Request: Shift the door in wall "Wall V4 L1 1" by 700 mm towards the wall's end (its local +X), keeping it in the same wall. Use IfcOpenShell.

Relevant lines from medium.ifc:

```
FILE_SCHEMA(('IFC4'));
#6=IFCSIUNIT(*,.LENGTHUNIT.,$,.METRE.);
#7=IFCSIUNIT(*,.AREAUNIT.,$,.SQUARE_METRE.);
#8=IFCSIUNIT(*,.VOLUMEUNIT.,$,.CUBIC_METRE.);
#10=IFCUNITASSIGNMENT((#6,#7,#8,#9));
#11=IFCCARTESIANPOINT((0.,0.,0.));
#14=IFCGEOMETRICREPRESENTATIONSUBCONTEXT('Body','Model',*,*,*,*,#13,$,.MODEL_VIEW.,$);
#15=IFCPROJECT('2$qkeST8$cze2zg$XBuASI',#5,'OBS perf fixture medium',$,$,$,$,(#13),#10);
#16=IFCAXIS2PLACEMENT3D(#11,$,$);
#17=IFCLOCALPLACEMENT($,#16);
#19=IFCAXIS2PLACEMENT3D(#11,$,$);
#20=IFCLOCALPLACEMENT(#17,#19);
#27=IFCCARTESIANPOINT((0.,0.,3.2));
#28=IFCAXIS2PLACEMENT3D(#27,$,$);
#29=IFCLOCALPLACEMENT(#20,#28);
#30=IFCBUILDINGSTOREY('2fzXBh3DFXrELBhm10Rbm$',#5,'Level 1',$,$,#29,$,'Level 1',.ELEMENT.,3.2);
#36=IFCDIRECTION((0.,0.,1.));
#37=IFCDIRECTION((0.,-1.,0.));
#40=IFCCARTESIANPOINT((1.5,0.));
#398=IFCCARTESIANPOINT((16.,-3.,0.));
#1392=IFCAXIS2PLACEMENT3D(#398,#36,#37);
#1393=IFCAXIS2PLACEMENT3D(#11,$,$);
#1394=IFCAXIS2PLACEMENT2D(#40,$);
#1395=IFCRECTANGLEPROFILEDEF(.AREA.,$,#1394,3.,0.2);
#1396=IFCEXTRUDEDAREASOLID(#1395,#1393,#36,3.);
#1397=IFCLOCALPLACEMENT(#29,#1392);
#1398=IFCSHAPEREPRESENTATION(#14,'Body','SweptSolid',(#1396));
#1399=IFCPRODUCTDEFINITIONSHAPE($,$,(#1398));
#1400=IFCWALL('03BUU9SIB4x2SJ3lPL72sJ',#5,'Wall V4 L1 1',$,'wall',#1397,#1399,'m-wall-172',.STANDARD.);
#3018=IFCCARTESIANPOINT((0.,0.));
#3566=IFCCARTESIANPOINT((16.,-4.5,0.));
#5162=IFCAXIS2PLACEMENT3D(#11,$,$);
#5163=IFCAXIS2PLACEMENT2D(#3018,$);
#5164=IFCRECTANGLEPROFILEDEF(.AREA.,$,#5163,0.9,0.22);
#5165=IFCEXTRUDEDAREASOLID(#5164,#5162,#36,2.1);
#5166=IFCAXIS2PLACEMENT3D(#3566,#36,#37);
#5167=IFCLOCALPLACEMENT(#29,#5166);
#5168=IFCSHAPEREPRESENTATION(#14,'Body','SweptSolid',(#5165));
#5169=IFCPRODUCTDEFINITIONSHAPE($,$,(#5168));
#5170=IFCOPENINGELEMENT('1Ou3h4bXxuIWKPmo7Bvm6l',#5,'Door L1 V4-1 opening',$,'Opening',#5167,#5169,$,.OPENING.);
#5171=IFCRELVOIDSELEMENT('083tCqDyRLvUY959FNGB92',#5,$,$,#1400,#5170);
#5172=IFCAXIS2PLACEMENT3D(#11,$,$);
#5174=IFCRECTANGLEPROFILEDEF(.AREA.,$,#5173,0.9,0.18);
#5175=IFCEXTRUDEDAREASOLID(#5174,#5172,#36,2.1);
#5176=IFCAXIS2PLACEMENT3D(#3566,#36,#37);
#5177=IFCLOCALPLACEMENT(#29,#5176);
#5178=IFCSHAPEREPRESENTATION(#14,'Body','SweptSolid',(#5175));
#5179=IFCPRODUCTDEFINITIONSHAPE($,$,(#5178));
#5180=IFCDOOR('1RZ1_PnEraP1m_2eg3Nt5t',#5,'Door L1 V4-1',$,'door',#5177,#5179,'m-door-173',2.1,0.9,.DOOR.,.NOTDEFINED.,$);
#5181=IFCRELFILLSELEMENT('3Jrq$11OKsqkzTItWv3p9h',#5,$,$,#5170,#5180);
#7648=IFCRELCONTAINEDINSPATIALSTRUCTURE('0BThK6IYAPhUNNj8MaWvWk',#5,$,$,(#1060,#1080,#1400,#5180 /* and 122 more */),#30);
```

```python
import ifcopenshell
import ifcopenshell.api.geometry
import ifcopenshell.util.placement

model = ifcopenshell.open("medium.ifc")

door = model.by_guid("1RZ1_PnEraP1m_2eg3Nt5t")
opening = door.FillsVoids[0].RelatingOpeningElement
wall = opening.VoidsElements[0].RelatingBuildingElement

wall_matrix = ifcopenshell.util.placement.get_local_placement(wall.ObjectPlacement)
shift = wall_matrix[:3, 0] * 0.7
before = ifcopenshell.util.placement.get_local_placement(door.ObjectPlacement)[:3, 3].copy()

# The door is not placed relative to its opening, so move both.
for product in (opening, door):
    matrix = ifcopenshell.util.placement.get_local_placement(product.ObjectPlacement)
    matrix[:3, 3] += shift
    ifcopenshell.api.geometry.edit_object_placement(model, product=product, matrix=matrix, is_si=False)

after = ifcopenshell.util.placement.get_local_placement(door.ObjectPlacement)[:3, 3]
print("door moved by", (after - before).round(3) + 0.0)

model.write("medium_v2.ifc")
```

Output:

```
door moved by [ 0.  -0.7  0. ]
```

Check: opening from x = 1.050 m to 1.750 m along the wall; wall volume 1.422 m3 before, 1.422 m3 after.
